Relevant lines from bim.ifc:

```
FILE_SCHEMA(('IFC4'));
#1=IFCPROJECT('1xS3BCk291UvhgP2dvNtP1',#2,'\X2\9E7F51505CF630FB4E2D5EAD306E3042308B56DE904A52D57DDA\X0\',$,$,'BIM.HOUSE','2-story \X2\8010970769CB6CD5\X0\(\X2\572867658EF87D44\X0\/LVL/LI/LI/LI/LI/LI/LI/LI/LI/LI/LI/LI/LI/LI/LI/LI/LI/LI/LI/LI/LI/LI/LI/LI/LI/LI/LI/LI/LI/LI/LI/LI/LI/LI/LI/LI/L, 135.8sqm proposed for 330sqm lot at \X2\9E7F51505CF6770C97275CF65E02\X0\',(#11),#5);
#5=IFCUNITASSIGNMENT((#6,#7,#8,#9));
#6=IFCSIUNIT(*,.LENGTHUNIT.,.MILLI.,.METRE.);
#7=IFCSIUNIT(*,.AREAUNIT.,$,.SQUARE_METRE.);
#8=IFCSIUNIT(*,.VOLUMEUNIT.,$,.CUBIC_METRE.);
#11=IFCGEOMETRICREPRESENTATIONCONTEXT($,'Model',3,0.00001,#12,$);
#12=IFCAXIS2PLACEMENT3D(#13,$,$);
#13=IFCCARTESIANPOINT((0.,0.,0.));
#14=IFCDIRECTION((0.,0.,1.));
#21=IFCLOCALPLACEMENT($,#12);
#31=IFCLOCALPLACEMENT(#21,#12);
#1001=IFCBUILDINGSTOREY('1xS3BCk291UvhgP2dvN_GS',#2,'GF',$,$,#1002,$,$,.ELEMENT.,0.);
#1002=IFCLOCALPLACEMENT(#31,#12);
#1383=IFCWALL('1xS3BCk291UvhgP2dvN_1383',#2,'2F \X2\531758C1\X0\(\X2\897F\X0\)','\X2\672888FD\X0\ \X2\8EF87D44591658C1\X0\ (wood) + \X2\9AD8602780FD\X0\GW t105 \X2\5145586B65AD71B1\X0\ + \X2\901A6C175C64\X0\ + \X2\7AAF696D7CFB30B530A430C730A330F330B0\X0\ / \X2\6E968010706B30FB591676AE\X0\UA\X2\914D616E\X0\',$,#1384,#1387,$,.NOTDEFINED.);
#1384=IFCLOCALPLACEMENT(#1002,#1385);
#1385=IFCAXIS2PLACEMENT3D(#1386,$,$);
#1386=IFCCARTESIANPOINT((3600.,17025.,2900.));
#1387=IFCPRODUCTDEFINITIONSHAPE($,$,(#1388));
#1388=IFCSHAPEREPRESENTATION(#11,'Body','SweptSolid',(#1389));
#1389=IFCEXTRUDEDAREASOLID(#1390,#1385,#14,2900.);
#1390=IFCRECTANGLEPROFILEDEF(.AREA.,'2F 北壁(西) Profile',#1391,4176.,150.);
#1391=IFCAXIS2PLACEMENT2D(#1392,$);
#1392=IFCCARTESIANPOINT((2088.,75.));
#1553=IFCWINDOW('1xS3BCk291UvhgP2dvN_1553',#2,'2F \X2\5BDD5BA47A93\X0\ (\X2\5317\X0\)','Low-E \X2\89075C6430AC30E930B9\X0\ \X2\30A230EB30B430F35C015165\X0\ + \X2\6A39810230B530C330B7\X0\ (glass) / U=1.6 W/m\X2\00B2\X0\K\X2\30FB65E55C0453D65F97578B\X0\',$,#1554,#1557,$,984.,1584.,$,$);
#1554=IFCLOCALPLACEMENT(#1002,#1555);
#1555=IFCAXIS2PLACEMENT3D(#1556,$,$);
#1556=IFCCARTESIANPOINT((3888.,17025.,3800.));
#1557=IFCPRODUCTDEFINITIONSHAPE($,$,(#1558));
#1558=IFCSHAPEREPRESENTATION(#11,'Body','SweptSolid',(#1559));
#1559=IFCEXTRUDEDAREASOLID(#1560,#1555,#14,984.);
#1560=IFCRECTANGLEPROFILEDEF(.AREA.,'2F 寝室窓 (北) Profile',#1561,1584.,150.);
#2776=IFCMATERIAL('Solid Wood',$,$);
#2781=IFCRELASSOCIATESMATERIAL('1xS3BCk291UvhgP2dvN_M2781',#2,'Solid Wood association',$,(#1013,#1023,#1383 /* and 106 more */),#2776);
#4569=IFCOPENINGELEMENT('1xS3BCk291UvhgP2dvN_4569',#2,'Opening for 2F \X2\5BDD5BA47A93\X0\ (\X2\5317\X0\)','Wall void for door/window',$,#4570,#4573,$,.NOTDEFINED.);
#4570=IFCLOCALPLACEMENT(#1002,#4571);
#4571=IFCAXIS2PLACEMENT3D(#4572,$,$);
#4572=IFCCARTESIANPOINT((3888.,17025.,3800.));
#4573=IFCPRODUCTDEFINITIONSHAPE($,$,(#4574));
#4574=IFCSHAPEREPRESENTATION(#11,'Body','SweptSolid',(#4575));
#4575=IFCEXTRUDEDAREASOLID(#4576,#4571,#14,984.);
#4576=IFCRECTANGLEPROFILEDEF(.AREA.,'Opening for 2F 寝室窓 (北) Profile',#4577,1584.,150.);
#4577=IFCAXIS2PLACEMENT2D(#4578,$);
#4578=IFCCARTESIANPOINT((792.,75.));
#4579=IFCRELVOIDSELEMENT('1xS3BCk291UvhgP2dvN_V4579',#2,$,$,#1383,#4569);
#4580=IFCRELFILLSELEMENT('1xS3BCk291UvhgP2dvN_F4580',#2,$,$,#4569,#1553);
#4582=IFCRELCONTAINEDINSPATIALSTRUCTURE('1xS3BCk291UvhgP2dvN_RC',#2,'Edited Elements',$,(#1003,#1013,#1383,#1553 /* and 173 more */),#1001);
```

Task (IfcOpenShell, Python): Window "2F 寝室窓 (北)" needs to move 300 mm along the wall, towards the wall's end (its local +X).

```python
import ifcopenshell
import ifcopenshell.api.geometry
import ifcopenshell.util.placement
import ifcopenshell.util.unit

model = ifcopenshell.open("bim.ifc")
unit_scale = ifcopenshell.util.unit.calculate_unit_scale(model)

window = model.by_guid("1xS3BCk291UvhgP2dvN_1553")
opening = window.FillsVoids[0].RelatingOpeningElement
wall = opening.VoidsElements[0].RelatingBuildingElement

wall_matrix = ifcopenshell.util.placement.get_local_placement(wall.ObjectPlacement)
shift = wall_matrix[:3, 0] * 0.3 / unit_scale
before = ifcopenshell.util.placement.get_local_placement(window.ObjectPlacement)[:3, 3].copy()

# The window is not placed relative to its opening, so move both.
for product in (opening, window):
    matrix = ifcopenshell.util.placement.get_local_placement(product.ObjectPlacement)
    matrix[:3, 3] += shift
    ifcopenshell.api.geometry.edit_object_placement(model, product=product, matrix=matrix, is_si=False)

after = ifcopenshell.util.placement.get_local_placement(window.ObjectPlacement)[:3, 3]
print("window moved by", (after - before).round(3) + 0.0)

model.write("bim_v2.ifc")
```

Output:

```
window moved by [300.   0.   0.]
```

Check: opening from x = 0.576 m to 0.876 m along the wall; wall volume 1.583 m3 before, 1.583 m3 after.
